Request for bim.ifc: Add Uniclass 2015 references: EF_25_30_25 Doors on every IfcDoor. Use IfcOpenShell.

First a look at what the model holds.

```python
import ifcopenshell

model = ifcopenshell.open("bim.ifc")
print(model.schema)
print("classifications:", [c.Name for c in model.by_type("IfcClassification")])
for ifc_class in ("IfcDoor", "IfcRoof", "IfcStair", "IfcWall", "IfcWindow"):
    print(ifc_class, len(model.by_type(ifc_class)))
```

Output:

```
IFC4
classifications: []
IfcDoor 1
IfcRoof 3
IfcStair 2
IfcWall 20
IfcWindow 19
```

```python
import ifcopenshell
import ifcopenshell.api.classification

model = ifcopenshell.open("bim.ifc")

system = ifcopenshell.api.classification.add_classification(model, classification="Uniclass 2015")

codes = {
    "IfcDoor": ("EF_25_30_25", "Doors"),
}
for ifc_class, (code, name) in codes.items():
    products = model.by_type(ifc_class)
    ifcopenshell.api.classification.add_reference(
        model, products=products, classification=system, identification=code, name=name
    )
    print(code, len(products))

model.write("bim_rev.ifc")
```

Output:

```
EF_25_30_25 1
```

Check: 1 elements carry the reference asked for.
